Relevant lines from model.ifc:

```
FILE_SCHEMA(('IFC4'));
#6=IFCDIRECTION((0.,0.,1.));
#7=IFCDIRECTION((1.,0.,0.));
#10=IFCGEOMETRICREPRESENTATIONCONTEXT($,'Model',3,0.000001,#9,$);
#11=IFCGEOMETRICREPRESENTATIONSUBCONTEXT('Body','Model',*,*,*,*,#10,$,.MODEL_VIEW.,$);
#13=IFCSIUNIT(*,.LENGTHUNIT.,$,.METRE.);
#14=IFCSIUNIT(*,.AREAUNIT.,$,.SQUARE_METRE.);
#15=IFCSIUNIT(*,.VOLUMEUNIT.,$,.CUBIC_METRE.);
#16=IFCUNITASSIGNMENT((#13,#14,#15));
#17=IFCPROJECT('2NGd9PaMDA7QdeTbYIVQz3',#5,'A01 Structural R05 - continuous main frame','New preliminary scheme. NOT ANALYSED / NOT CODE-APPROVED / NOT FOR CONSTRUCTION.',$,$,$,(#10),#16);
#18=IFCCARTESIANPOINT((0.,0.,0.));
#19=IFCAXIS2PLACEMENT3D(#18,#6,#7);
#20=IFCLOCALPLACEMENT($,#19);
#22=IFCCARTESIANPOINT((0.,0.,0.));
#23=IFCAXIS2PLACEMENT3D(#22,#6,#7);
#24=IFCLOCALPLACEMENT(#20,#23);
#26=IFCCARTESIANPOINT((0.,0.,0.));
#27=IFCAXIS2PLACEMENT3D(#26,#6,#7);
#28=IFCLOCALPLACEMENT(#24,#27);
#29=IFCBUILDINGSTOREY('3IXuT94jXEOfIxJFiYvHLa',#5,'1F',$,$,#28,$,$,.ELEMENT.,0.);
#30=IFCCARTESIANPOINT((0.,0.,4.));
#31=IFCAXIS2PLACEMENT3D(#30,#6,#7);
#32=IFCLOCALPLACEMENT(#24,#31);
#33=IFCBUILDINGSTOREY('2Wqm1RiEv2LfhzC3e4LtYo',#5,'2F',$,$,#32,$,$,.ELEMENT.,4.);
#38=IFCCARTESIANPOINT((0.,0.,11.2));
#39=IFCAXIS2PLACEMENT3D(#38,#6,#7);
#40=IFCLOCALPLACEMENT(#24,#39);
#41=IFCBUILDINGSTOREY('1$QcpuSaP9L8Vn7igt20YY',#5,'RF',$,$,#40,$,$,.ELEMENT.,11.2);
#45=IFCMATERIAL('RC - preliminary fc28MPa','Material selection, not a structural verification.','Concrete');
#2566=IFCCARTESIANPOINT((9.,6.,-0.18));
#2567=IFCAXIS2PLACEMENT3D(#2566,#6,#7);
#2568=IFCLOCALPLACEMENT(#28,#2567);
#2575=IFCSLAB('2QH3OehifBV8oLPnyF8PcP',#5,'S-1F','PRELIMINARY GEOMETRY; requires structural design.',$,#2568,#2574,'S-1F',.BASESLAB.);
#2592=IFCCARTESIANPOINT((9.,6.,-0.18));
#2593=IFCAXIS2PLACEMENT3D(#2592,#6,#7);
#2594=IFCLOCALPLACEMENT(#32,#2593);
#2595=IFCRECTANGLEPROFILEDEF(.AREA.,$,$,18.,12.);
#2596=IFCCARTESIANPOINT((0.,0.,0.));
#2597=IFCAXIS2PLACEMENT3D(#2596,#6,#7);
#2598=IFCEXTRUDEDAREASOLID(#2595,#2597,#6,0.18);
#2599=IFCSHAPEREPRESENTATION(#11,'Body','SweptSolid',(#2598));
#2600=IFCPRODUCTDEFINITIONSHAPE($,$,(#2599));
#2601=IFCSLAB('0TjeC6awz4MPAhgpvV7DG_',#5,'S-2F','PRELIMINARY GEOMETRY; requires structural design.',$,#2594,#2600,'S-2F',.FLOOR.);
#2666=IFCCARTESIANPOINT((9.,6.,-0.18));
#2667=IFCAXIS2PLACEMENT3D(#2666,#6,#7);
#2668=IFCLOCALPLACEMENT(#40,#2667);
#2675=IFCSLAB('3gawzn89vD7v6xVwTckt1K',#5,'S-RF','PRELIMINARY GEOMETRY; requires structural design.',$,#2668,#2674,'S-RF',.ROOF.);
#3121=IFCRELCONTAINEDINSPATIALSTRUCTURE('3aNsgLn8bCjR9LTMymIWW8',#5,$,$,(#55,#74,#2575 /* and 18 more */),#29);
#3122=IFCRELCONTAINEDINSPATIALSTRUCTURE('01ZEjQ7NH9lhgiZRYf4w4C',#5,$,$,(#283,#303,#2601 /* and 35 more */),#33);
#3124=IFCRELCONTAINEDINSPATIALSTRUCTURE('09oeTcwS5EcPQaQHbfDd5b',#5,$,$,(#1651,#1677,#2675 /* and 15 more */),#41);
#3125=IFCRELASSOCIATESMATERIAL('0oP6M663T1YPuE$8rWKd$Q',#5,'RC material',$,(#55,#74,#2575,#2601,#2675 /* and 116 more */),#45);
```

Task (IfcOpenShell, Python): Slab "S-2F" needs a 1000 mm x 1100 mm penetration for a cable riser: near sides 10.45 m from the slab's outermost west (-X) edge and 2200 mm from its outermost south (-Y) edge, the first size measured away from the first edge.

```python
import numpy as np
import ifcopenshell
import ifcopenshell.api.feature
import ifcopenshell.api.geometry
import ifcopenshell.api.root
import ifcopenshell.geom
import ifcopenshell.util.placement
import ifcopenshell.util.representation
import ifcopenshell.util.shape
import ifcopenshell.util.unit

model = ifcopenshell.open("model.ifc")
unit_scale = ifcopenshell.util.unit.calculate_unit_scale(model)
settings = ifcopenshell.geom.settings()


def volume(element):
    """Net volume in cubic metres, openings subtracted."""
    shape = ifcopenshell.geom.create_shape(settings, element)
    return ifcopenshell.util.shape.get_volume(shape.geometry)


slab = model.by_guid("0TjeC6awz4MPAhgpvV7DG_")
before = volume(slab)

# Extent in the slab's own axes, in metres. The edges named are its -X and -Y sides.
slab_shape = ifcopenshell.geom.create_shape(settings, slab)
vertices = ifcopenshell.util.shape.get_vertices(slab_shape.geometry)
x_min, y_min, bottom = vertices.min(axis=0)
top = vertices[:, 2].max()

opening = ifcopenshell.api.root.create_entity(model, ifc_class="IfcOpeningElement", name="Cable riser opening", predefined_type="OPENING")
context = ifcopenshell.util.representation.get_context(model, "Model", "Body", "MODEL_VIEW")
width, depth = 1, 1.1
outline = [(0.0, 0.0), (width, 0.0), (width, depth), (0.0, depth), (0.0, 0.0)]
# Overshoot both faces by 50 mm so the cut is clean.
shape = ifcopenshell.api.geometry.add_slab_representation(
    model, context=context, depth=top - bottom + 0.1, polyline=outline
)
ifcopenshell.api.geometry.assign_representation(model, product=opening, representation=shape)

matrix = ifcopenshell.util.placement.get_local_placement(slab.ObjectPlacement)
matrix[:, 3] = matrix @ np.append(np.array([x_min + 10.45, y_min + 2.2, bottom - 0.05]) / unit_scale, 1.0)
ifcopenshell.api.geometry.edit_object_placement(model, product=opening, matrix=matrix, is_si=False)
ifcopenshell.api.feature.add_feature(model, feature=opening, element=slab)

after = volume(slab)

print(f"slab volume {before:.3f} -> {after:.3f} m3")

model.write("model-out.ifc")
```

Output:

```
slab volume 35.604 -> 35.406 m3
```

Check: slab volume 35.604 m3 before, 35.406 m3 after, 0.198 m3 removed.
